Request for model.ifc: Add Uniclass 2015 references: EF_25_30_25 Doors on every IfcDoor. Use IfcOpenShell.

First a look at what the model holds.

```python
import ifcopenshell

model = ifcopenshell.open("model.ifc")
print(model.schema)
print("classifications:", [c.Name for c in model.by_type("IfcClassification")])
for ifc_class in ("IfcDoor", "IfcRoof", "IfcStair", "IfcWall", "IfcWindow"):
    print(ifc_class, len(model.by_type(ifc_class)))
```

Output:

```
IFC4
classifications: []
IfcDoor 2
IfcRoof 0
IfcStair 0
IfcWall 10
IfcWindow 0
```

```python
import ifcopenshell
import ifcopenshell.api.classification

model = ifcopenshell.open("model.ifc")

system = ifcopenshell.api.classification.add_classification(model, classification="Uniclass 2015")

codes = {
    "IfcDoor": ("EF_25_30_25", "Doors"),
}
for ifc_class, (code, name) in codes.items():
    products = model.by_type(ifc_class)
    ifcopenshell.api.classification.add_reference(
        model, products=products, classification=system, identification=code, name=name
    )
    print(code, len(products))

model.write("model_updated.ifc")
```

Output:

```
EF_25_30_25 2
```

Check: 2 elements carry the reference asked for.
